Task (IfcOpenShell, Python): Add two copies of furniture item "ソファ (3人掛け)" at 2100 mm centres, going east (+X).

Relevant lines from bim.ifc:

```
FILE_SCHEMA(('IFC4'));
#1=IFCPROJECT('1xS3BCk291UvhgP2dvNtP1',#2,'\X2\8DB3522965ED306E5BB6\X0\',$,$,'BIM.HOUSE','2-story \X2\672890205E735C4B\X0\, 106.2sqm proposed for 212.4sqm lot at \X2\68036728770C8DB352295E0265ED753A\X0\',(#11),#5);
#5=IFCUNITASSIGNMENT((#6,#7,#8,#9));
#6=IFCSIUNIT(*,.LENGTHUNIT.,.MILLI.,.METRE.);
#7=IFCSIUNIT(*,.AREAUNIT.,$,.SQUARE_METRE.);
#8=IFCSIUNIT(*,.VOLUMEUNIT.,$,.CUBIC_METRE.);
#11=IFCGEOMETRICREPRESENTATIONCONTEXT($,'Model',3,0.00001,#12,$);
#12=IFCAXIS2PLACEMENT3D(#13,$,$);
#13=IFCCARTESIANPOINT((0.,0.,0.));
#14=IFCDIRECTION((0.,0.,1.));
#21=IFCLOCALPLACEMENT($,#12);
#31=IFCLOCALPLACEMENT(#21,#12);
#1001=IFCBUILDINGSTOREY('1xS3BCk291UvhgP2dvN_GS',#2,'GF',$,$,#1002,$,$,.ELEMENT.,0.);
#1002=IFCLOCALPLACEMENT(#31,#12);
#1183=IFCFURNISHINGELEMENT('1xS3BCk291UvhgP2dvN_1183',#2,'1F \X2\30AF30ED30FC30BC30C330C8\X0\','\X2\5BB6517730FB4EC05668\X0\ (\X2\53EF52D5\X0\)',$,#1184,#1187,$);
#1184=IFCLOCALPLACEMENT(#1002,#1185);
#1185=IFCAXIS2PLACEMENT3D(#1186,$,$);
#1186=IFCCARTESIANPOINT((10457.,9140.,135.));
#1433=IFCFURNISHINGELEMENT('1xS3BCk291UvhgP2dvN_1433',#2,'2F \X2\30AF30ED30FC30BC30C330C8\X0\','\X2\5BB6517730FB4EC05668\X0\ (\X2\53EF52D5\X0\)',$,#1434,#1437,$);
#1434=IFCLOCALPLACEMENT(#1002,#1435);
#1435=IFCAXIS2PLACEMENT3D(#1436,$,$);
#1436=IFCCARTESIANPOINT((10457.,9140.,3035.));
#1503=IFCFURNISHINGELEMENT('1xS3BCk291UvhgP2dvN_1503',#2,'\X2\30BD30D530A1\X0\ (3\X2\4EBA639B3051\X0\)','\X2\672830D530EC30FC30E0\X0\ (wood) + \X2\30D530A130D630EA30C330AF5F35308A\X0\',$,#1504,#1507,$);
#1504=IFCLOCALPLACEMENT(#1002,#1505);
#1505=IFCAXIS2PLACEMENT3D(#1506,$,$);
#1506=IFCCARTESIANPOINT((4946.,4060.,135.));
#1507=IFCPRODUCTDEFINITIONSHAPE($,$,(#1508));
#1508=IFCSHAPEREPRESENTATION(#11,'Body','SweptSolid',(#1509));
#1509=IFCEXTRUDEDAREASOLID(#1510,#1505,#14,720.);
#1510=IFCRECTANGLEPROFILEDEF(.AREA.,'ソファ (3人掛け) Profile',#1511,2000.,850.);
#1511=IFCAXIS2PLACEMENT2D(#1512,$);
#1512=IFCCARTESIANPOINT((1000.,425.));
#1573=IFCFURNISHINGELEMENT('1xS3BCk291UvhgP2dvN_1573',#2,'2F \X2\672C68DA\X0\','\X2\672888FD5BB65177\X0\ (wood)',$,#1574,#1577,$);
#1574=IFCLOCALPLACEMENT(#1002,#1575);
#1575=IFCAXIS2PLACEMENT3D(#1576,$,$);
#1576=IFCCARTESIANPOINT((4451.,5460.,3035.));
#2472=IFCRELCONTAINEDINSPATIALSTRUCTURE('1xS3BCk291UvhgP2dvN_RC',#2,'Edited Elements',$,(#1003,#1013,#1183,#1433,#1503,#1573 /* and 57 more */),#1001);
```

```python
import numpy as np
import ifcopenshell
import ifcopenshell.api.geometry
import ifcopenshell.api.root
import ifcopenshell.util.element
import ifcopenshell.util.placement
import ifcopenshell.util.unit

model = ifcopenshell.open("bim.ifc")
unit_scale = ifcopenshell.util.unit.calculate_unit_scale(model)


def reuse_history(source, copy):
    """copy_class also copies each property set's owner history, people and application; keep the originals."""
    for rel in copy.IsDefinedBy:
        if rel.is_a("IfcRelDefinesByProperties") and (history := rel.RelatingPropertyDefinition.OwnerHistory):
            rel.RelatingPropertyDefinition.OwnerHistory = source.OwnerHistory
            ifcopenshell.util.element.remove_deep2(model, history)


source = model.by_guid("1xS3BCk291UvhgP2dvN_1503")
base = ifcopenshell.util.placement.get_local_placement(source.ObjectPlacement)
step = np.array([1.0, 0.0, 0.0]) * 2.1 / unit_scale

for i in range(1, 3):
    copy = ifcopenshell.api.root.copy_class(model, product=source)
    copy.Representation = ifcopenshell.util.element.copy_deep(
        model, source.Representation, exclude=["IfcGeometricRepresentationContext", "IfcRepresentationMap"]
    )
    reuse_history(source, copy)
    matrix = base.copy()
    matrix[:3, 3] += i * step
    print("added at", matrix[:3, 3].round(3) + 0.0)
    ifcopenshell.api.geometry.edit_object_placement(model, product=copy, matrix=matrix, is_si=False)

model.write("bim_edited.ifc")
```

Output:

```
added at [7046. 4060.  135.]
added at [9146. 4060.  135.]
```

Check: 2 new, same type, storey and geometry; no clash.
